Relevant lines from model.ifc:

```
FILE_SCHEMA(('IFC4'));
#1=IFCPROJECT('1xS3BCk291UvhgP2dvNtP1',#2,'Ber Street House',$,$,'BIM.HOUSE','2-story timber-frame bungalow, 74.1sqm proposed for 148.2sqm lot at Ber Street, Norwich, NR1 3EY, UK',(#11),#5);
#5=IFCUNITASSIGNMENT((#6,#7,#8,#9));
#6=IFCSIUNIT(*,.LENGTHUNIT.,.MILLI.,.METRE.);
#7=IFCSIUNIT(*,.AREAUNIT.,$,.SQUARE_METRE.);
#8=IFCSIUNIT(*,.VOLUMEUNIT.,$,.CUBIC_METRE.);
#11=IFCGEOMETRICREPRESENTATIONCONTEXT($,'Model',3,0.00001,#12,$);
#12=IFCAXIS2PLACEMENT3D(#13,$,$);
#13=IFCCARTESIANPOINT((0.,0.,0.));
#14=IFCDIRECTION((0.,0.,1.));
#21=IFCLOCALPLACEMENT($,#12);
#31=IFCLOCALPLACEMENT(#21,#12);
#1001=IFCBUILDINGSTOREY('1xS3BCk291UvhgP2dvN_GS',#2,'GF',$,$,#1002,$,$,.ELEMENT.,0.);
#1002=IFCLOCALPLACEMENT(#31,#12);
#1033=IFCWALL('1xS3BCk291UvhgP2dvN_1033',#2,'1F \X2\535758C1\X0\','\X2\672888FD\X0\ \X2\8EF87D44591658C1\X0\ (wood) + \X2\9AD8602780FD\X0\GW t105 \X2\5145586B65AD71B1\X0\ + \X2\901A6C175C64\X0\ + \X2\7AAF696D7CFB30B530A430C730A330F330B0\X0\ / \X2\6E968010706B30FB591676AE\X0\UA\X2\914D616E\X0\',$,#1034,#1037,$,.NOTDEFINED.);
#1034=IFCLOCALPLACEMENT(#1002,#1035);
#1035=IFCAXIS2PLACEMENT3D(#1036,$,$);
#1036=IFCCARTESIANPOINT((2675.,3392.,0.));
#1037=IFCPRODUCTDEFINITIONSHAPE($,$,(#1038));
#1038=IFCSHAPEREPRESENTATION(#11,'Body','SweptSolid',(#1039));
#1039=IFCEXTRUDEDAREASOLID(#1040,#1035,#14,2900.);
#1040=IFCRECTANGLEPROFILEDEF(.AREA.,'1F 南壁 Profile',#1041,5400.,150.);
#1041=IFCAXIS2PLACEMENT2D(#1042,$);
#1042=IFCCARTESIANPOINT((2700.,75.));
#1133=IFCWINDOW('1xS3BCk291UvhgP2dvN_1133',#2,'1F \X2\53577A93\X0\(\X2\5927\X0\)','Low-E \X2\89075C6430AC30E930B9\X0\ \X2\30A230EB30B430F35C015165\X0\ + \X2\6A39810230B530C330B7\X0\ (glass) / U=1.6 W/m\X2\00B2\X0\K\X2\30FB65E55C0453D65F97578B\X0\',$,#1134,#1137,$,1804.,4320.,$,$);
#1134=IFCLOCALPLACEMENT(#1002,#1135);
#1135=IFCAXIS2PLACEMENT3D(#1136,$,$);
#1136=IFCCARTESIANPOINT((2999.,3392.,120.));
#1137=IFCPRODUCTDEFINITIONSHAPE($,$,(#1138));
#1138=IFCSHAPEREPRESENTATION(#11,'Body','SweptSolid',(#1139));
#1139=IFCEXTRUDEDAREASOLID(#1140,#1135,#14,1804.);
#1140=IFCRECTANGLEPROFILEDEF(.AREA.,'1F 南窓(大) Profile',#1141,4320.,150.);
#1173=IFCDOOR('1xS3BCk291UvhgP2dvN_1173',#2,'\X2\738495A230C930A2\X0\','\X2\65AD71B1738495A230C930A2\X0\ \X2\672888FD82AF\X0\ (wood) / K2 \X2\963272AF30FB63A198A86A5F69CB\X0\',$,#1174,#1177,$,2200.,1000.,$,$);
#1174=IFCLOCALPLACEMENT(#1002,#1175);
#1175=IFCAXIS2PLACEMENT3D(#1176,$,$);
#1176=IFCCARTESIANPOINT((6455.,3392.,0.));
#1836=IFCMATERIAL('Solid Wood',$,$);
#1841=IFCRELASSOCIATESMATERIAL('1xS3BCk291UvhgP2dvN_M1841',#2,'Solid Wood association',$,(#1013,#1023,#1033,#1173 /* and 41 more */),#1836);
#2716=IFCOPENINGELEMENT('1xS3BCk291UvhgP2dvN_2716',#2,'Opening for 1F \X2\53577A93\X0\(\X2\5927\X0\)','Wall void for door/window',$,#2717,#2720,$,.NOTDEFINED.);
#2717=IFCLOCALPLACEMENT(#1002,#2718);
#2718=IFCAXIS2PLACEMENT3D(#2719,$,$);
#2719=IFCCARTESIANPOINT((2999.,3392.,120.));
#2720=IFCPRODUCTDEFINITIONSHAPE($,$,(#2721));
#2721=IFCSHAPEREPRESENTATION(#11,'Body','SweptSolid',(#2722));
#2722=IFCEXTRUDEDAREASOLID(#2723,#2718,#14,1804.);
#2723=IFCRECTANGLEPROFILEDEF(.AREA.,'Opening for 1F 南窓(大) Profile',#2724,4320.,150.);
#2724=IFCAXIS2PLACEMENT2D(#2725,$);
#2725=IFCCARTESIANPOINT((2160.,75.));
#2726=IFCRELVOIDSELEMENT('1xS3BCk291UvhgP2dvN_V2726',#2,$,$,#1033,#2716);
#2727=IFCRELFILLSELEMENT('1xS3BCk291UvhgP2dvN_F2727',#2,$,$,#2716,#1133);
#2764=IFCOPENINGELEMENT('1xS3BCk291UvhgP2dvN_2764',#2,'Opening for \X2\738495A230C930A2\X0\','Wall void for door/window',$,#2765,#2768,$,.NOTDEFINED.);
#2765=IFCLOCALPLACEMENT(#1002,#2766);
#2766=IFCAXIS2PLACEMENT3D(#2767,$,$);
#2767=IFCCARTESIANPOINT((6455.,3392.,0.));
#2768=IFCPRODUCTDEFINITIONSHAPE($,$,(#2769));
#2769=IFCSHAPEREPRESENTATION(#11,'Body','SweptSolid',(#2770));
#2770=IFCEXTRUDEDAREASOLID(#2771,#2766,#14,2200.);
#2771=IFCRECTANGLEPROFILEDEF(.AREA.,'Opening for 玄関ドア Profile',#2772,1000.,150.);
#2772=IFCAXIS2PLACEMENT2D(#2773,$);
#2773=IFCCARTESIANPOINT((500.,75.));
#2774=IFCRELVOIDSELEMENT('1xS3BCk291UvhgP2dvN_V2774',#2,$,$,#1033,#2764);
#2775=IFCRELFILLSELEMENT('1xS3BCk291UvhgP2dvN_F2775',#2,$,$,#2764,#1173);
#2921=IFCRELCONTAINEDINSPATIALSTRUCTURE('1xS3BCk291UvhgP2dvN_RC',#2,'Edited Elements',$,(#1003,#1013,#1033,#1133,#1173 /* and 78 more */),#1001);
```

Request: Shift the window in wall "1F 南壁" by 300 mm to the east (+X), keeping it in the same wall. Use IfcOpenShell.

```python
import ifcopenshell
import ifcopenshell.api.geometry
import ifcopenshell.util.placement
import ifcopenshell.util.unit

model = ifcopenshell.open("model.ifc")
unit_scale = ifcopenshell.util.unit.calculate_unit_scale(model)

window = model.by_guid("1xS3BCk291UvhgP2dvN_1133")
opening = window.FillsVoids[0].RelatingOpeningElement
wall = opening.VoidsElements[0].RelatingBuildingElement

wall_matrix = ifcopenshell.util.placement.get_local_placement(wall.ObjectPlacement)
shift = wall_matrix[:3, 0] * 0.3 / unit_scale
before = ifcopenshell.util.placement.get_local_placement(window.ObjectPlacement)[:3, 3].copy()

# The window is not placed relative to its opening, so move both.
for product in (opening, window):
    matrix = ifcopenshell.util.placement.get_local_placement(product.ObjectPlacement)
    matrix[:3, 3] += shift
    ifcopenshell.api.geometry.edit_object_placement(model, product=product, matrix=matrix, is_si=False)

after = ifcopenshell.util.placement.get_local_placement(window.ObjectPlacement)[:3, 3]
print("window moved by", (after - before).round(3) + 0.0)

model.write("model-out.ifc")
```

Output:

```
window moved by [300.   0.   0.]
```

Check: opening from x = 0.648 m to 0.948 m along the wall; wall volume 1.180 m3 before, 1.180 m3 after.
